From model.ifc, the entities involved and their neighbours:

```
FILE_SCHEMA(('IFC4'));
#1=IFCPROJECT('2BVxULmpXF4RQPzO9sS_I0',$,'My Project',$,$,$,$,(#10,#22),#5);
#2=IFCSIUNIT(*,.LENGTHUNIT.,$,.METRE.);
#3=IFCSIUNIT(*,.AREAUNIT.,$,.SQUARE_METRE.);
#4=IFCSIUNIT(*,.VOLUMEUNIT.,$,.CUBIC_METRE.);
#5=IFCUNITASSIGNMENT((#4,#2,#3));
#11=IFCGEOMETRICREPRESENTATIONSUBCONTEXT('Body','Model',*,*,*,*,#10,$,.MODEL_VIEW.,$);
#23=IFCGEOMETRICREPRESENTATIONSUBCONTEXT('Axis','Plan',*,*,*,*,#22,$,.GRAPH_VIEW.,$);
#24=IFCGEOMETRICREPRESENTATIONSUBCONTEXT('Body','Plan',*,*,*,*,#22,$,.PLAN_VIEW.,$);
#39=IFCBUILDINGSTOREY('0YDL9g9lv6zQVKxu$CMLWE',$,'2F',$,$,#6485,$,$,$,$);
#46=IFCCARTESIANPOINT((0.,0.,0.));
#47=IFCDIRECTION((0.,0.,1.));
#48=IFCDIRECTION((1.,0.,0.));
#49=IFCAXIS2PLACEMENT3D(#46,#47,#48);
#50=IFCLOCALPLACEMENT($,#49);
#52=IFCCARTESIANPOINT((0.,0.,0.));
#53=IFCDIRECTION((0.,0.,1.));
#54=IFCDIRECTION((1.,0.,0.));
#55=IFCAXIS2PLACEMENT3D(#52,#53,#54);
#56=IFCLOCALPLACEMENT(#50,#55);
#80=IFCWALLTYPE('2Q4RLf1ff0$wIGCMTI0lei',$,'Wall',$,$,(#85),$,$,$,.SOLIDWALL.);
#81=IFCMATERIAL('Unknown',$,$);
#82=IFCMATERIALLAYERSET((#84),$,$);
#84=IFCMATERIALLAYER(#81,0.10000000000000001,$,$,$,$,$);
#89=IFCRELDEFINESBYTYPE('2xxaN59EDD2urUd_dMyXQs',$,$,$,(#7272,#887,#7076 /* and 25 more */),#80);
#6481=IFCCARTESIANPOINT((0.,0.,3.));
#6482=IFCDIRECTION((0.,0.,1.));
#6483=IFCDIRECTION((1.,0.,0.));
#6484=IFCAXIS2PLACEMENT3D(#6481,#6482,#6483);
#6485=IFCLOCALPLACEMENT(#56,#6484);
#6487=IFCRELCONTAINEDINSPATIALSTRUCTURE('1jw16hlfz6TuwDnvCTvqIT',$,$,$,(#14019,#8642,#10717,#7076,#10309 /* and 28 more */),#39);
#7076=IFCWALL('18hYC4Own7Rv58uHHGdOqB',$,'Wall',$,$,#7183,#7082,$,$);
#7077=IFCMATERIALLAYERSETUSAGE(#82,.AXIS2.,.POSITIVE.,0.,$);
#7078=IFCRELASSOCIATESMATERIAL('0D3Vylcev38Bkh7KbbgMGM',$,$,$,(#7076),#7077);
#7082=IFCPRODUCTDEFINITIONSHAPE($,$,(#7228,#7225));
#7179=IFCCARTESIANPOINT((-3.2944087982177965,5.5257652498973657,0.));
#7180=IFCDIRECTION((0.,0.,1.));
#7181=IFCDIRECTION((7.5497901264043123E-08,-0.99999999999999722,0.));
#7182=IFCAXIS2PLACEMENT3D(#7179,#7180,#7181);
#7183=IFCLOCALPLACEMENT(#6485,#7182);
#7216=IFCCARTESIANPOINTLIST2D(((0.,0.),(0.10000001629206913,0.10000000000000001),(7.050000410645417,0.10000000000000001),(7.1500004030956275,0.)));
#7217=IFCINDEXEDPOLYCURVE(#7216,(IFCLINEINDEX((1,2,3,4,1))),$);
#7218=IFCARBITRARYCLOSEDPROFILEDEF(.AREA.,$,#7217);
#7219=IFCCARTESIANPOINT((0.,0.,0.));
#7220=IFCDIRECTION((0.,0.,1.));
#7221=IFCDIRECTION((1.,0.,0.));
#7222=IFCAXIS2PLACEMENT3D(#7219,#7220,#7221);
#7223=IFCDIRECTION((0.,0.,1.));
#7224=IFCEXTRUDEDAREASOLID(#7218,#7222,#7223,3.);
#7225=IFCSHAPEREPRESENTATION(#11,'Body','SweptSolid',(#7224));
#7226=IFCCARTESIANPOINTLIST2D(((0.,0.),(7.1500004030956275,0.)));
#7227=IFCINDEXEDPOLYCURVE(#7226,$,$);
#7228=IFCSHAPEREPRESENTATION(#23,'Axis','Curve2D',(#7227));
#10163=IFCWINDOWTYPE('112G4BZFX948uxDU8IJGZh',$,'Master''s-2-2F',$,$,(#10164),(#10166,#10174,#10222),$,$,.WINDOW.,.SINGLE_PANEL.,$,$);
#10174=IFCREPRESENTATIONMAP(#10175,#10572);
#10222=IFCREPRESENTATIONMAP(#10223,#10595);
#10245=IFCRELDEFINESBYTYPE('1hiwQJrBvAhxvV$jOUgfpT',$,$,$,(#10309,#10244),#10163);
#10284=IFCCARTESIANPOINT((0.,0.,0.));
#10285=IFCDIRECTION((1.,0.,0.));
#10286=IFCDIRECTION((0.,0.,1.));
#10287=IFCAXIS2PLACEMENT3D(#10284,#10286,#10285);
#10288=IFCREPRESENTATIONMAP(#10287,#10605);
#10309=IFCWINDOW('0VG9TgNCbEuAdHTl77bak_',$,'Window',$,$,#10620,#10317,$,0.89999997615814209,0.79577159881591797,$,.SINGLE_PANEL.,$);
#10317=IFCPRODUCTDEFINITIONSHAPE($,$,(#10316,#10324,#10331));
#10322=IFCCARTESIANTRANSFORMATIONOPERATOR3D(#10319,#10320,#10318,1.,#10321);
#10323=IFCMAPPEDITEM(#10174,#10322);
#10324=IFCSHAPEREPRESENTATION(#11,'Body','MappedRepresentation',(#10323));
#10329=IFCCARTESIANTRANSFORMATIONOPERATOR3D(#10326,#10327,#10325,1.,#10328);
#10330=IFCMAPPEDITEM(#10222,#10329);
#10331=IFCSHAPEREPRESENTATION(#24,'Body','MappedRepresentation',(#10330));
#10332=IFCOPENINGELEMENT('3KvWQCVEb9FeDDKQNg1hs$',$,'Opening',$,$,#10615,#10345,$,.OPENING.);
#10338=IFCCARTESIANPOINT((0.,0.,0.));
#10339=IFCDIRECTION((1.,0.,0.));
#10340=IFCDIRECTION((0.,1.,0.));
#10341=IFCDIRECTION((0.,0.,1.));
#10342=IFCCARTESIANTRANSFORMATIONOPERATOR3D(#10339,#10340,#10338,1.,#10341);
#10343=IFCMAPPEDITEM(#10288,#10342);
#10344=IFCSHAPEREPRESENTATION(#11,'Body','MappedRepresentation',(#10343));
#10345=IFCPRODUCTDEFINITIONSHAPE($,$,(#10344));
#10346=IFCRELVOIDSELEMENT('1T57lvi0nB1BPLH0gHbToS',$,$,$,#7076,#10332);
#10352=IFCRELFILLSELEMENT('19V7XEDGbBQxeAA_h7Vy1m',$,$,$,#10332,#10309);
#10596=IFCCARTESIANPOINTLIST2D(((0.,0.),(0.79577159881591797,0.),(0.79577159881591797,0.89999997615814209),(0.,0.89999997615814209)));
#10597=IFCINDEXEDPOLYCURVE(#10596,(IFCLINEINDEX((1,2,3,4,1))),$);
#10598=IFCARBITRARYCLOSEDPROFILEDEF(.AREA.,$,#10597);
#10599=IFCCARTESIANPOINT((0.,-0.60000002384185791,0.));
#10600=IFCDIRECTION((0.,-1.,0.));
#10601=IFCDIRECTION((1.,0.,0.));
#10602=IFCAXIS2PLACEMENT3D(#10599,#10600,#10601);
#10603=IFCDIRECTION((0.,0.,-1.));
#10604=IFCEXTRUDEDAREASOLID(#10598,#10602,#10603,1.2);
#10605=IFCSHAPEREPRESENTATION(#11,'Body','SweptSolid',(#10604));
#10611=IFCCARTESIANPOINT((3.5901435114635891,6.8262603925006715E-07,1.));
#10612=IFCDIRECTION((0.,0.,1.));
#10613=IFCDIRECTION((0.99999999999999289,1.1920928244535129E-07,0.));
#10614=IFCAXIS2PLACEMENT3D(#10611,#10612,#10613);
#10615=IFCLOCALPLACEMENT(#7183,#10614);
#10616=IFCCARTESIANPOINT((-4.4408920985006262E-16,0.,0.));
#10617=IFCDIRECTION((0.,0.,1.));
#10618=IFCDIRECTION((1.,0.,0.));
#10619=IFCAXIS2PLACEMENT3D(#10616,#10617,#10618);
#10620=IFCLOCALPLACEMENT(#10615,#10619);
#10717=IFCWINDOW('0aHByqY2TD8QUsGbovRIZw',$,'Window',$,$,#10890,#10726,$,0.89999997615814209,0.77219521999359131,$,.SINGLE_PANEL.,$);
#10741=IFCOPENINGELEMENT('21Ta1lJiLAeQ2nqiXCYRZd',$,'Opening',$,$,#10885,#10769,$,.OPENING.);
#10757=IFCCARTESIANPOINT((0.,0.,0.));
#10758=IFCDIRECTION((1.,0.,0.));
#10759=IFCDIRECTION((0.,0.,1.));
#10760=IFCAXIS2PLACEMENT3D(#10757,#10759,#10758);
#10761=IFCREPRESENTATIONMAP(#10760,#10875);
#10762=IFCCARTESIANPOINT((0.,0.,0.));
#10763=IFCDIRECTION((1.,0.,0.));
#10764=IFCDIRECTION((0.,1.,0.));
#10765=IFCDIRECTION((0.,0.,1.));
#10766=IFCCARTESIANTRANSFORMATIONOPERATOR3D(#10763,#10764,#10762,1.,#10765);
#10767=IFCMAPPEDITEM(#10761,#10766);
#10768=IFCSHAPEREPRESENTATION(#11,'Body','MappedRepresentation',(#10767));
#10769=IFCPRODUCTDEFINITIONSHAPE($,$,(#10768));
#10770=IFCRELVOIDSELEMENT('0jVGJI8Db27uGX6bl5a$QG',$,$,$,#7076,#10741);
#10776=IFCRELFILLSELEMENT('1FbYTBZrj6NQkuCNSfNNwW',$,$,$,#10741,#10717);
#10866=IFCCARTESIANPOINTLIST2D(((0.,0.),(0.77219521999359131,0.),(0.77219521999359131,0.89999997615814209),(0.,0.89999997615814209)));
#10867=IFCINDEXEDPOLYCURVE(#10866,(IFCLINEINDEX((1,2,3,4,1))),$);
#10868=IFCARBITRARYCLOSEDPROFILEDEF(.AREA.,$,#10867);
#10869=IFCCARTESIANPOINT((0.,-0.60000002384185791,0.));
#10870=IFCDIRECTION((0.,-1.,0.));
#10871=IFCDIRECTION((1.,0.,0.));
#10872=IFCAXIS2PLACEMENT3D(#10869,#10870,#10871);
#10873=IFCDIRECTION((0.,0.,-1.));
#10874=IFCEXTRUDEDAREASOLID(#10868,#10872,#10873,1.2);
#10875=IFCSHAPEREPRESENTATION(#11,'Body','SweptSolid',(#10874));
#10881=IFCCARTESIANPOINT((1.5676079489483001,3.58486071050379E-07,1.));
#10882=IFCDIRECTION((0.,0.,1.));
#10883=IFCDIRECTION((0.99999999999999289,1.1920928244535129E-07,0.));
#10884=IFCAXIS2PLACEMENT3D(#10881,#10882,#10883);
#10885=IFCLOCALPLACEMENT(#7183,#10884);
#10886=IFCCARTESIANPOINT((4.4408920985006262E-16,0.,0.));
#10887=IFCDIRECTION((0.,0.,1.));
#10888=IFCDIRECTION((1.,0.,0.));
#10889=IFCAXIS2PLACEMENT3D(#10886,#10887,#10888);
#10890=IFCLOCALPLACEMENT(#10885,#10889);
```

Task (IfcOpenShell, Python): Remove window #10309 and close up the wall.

```python
import ifcopenshell
import ifcopenshell.api.feature
import ifcopenshell.api.root
import ifcopenshell.geom
import ifcopenshell.util.shape

model = ifcopenshell.open("model.ifc")
settings = ifcopenshell.geom.settings()


def volume(element):
    """Net volume in cubic metres, openings subtracted."""
    shape = ifcopenshell.geom.create_shape(settings, element)
    return ifcopenshell.util.shape.get_volume(shape.geometry)


window = model.by_id(10309)
opening = window.FillsVoids[0].RelatingOpeningElement
wall = opening.VoidsElements[0].RelatingBuildingElement
before = volume(wall)

ifcopenshell.api.root.remove_product(model, product=window)
ifcopenshell.api.feature.remove_feature(model, feature=opening)

after = volume(wall)

print(f"wall volume {before:.3f} -> {after:.3f} m3")

model.write("model_edited.ifc")
```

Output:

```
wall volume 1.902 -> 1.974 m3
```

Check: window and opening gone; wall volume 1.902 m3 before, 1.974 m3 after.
